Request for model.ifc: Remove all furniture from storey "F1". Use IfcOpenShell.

First a look at what the model holds.

```python
import ifcopenshell
import ifcopenshell.util.element

model = ifcopenshell.open("model.ifc")
print(model.schema)
storey = next(s for s in model.by_type("IfcBuildingStorey") if s.Name == "F1")
furniture = [e for e in ifcopenshell.util.element.get_decomposition(storey) if e.is_a("IfcFurnishingElement")]
seen = {}
for e in furniture:
    element_type = ifcopenshell.util.element.get_type(e)
    name = element_type.Name if element_type not in (None, e) else None
    seen[name] = seen.get(name, 0) + 1
for name, count in sorted(seen.items(), key=str):
    print(count, "x", name)
```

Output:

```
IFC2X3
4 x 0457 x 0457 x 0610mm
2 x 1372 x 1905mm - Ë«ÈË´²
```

```python
import ifcopenshell
import ifcopenshell.api.root
import ifcopenshell.util.element

model = ifcopenshell.open("model.ifc")

storey = next(s for s in model.by_type("IfcBuildingStorey") if s.Name == "F1")
furniture = [e for e in ifcopenshell.util.element.get_decomposition(storey) if e.is_a("IfcFurnishingElement")]

for e in furniture:
    ifcopenshell.api.root.remove_product(model, product=e)
print(len(furniture), "removed")

model.write("model_updated.ifc")
```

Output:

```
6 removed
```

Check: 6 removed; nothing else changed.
